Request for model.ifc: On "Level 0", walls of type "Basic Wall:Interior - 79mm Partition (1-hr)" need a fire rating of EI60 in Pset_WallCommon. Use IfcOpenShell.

First a look at what the model holds.

```python
import ifcopenshell
import ifcopenshell.util.element

model = ifcopenshell.open("model.ifc")
print(model.schema)
storey = next(s for s in model.by_type("IfcBuildingStorey") if s.Name == "Level 0")
walls = [e for e in ifcopenshell.util.element.get_decomposition(storey) if e.is_a("IfcWall")]
seen = {}
for e in walls:
    element_type = ifcopenshell.util.element.get_type(e)
    key = (element_type.Name if element_type != e and element_type else None, ifcopenshell.util.element.get_pset(e, "Pset_WallCommon", "FireRating"))
    seen[key] = seen.get(key, 0) + 1
for (name, value), count in sorted(seen.items(), key=str):
    print(count, "x", name, "|", value)
```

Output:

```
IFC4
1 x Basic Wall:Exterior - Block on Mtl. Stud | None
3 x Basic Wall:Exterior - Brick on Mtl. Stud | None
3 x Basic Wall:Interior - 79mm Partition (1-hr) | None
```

```python
import ifcopenshell
import ifcopenshell.api.pset
import ifcopenshell.util.element

model = ifcopenshell.open("model.ifc")

storey = next(s for s in model.by_type("IfcBuildingStorey") if s.Name == "Level 0")
walls = [e for e in ifcopenshell.util.element.get_decomposition(storey) if e.is_a("IfcWall")]

count = 0
for e in walls:
    element_type = ifcopenshell.util.element.get_type(e)
    if element_type in (None, e) or element_type.Name != "Basic Wall:Interior - 79mm Partition (1-hr)":
        continue
    # add_pset returns the element's existing set when there is one.
    pset = ifcopenshell.api.pset.add_pset(model, product=e, name="Pset_WallCommon")
    ifcopenshell.api.pset.edit_pset(model, pset=pset, properties={"FireRating": "EI60"})
    count += 1

print(count, "walls updated")

model.write("model-out.ifc")
```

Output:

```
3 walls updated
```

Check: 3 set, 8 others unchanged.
